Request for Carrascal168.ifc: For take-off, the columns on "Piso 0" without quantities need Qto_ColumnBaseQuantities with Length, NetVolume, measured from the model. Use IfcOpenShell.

First a look at what the model holds.

```python
import ifcopenshell
import ifcopenshell.util.element
import ifcopenshell.util.unit

model = ifcopenshell.open("Carrascal168.ifc")
print(model.schema)
for unit_type in ("LENGTHUNIT", "AREAUNIT", "VOLUMEUNIT"):
    print(unit_type, ifcopenshell.util.unit.calculate_unit_scale(model, unit_type))
storey = next(s for s in model.by_type("IfcBuildingStorey") if s.Name == "Piso 0")
columns = [e for e in ifcopenshell.util.element.get_decomposition(storey) if e.is_a("IfcColumn")]
for e in sorted(columns, key=lambda e: e.id()):
    print(e.id(), e.is_a(), e.Name, list(ifcopenshell.util.element.get_psets(e, qtos_only=True)), sep=" | ")
```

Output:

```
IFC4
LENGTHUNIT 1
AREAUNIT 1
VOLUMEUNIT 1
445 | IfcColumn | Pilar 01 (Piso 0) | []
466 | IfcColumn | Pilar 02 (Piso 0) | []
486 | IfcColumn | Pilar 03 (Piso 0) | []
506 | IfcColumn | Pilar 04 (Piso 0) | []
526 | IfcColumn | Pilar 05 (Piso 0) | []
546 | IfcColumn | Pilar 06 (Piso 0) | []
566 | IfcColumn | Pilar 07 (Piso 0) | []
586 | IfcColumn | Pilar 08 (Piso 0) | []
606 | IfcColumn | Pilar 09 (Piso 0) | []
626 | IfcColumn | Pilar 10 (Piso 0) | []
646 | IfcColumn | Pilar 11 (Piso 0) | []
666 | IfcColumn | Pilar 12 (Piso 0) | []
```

```python
import ifcopenshell
import ifcopenshell.api.pset
import ifcopenshell.geom
import ifcopenshell.util.element
import ifcopenshell.util.shape
import ifcopenshell.util.unit

model = ifcopenshell.open("Carrascal168.ifc")
unit_scale = ifcopenshell.util.unit.calculate_unit_scale(model)
volume_scale = ifcopenshell.util.unit.calculate_unit_scale(model, "VOLUMEUNIT")
settings = ifcopenshell.geom.settings()

storey = next(s for s in model.by_type("IfcBuildingStorey") if s.Name == "Piso 0")
columns = [e for e in ifcopenshell.util.element.get_decomposition(storey) if e.is_a("IfcColumn")]

for e in sorted(columns, key=lambda e: e.id()):
    if ifcopenshell.util.element.get_psets(e, qtos_only=True, should_inherit=False):
        continue
    # Geometry comes back in metres, in the element's own axes.
    shape = ifcopenshell.geom.create_shape(settings, e)
    values = {
        "Length": ifcopenshell.util.shape.get_z(shape.geometry) / unit_scale,
        "NetVolume": ifcopenshell.util.shape.get_volume(shape.geometry) / volume_scale,
    }
    qto = ifcopenshell.api.pset.add_qto(model, product=e, name="Qto_ColumnBaseQuantities")
    ifcopenshell.api.pset.edit_qto(model, qto=qto, properties=values)
    print(e.id(), {k: round(v, 3) for k, v in values.items()})

model.write("Carrascal168-out.ifc")
```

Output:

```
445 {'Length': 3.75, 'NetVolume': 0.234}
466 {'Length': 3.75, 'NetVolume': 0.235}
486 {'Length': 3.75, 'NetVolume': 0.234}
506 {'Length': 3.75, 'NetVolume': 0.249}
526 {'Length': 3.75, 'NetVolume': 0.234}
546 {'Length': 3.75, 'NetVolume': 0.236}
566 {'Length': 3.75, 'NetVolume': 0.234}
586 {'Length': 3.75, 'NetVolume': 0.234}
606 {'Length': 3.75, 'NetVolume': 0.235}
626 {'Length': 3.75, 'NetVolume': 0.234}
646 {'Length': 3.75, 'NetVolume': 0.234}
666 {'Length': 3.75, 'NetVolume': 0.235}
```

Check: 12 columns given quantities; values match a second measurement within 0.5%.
